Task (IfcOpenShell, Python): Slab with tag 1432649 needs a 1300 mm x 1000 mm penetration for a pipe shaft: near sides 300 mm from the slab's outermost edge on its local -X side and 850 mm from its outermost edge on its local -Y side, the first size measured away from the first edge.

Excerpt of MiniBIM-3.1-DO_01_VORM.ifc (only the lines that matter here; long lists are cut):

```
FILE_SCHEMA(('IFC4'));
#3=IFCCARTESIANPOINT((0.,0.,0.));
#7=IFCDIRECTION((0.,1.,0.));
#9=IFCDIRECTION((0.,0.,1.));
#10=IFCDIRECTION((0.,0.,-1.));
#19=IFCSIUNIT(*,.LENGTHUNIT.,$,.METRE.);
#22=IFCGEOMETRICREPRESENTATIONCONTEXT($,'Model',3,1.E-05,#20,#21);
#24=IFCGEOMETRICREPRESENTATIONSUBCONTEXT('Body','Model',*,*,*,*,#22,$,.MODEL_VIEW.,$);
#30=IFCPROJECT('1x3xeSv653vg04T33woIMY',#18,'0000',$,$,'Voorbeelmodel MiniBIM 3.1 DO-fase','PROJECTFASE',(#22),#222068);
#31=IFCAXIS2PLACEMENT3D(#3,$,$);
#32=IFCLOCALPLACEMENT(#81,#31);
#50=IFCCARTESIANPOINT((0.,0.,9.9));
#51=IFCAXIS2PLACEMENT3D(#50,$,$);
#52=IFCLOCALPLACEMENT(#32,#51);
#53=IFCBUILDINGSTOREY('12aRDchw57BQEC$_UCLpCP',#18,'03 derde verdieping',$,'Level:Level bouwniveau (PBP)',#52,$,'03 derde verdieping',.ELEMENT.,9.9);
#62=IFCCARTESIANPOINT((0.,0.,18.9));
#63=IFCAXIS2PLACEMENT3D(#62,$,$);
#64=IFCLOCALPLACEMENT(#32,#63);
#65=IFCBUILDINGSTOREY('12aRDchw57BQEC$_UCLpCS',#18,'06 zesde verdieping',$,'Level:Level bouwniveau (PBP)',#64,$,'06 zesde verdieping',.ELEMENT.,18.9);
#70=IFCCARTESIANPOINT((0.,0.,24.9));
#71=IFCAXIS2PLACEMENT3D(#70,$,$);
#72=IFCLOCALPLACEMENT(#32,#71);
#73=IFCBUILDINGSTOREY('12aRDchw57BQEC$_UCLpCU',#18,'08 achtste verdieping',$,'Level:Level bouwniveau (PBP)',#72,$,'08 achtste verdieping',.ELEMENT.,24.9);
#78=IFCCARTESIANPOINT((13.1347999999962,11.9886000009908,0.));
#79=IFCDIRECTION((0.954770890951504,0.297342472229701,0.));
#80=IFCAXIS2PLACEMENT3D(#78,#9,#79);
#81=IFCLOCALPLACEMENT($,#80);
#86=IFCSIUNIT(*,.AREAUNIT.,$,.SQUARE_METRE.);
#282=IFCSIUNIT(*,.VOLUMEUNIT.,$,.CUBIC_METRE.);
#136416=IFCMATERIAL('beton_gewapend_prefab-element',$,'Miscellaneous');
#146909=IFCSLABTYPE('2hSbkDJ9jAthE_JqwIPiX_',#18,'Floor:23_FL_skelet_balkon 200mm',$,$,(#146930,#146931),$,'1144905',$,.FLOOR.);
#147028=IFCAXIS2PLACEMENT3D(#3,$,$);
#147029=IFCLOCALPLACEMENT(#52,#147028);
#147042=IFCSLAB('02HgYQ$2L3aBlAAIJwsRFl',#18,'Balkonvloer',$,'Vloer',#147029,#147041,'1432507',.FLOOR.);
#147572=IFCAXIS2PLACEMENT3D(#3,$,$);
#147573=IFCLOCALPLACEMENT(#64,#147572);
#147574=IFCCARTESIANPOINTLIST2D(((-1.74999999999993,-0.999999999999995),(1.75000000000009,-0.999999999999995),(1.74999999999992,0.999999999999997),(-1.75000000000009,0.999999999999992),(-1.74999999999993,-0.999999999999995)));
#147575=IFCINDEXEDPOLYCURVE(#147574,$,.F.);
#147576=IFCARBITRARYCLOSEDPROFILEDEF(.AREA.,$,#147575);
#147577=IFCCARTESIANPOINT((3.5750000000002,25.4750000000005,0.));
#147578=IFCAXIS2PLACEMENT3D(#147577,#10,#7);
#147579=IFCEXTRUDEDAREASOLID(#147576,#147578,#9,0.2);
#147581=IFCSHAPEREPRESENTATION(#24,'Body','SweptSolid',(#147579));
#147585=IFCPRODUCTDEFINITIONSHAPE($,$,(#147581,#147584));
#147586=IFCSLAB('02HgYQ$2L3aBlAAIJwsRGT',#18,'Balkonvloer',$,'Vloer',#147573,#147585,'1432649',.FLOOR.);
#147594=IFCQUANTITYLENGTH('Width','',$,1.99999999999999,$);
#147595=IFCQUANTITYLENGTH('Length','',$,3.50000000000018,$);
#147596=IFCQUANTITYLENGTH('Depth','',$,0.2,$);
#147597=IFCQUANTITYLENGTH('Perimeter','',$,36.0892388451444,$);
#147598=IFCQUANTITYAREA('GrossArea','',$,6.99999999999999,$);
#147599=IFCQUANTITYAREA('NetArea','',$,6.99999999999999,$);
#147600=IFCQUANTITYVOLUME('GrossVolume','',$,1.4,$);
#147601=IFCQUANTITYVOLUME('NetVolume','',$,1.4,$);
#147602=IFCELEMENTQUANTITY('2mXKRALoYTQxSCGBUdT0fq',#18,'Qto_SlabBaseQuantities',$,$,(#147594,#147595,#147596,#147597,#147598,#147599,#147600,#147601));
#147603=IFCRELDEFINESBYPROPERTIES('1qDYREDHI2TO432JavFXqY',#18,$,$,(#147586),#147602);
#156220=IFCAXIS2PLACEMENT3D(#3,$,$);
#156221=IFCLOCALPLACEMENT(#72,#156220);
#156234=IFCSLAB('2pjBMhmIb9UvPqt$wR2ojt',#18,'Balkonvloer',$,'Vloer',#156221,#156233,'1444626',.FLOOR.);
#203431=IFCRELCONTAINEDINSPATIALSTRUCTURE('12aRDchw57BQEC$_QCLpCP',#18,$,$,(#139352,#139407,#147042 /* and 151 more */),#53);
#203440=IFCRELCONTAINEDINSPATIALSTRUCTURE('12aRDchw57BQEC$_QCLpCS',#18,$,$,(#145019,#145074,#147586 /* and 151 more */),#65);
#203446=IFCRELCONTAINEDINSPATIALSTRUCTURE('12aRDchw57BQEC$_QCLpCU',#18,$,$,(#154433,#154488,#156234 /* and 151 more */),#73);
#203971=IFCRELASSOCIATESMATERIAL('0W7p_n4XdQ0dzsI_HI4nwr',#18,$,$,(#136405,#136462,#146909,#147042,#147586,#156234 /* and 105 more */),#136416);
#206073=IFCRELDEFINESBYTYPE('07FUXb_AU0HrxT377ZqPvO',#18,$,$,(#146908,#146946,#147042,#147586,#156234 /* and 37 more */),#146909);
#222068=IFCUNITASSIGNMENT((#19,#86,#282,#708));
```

```python
import numpy as np
import ifcopenshell
import ifcopenshell.api.feature
import ifcopenshell.api.geometry
import ifcopenshell.api.pset
import ifcopenshell.api.root
import ifcopenshell.geom
import ifcopenshell.util.element
import ifcopenshell.util.placement
import ifcopenshell.util.representation
import ifcopenshell.util.shape
import ifcopenshell.util.unit

model = ifcopenshell.open("MiniBIM-3.1-DO_01_VORM.ifc")
unit_scale = ifcopenshell.util.unit.calculate_unit_scale(model)
area_scale = ifcopenshell.util.unit.calculate_unit_scale(model, "AREAUNIT")
volume_scale = ifcopenshell.util.unit.calculate_unit_scale(model, "VOLUMEUNIT")
settings = ifcopenshell.geom.settings()


def volume(element):
    """Net volume in cubic metres, openings subtracted."""
    shape = ifcopenshell.geom.create_shape(settings, element)
    return ifcopenshell.util.shape.get_volume(shape.geometry)


slab = model.by_guid("02HgYQ$2L3aBlAAIJwsRGT")
before = volume(slab)

# Extent in the slab's own axes, in metres. The edges named are its -X and -Y sides.
slab_shape = ifcopenshell.geom.create_shape(settings, slab)
vertices = ifcopenshell.util.shape.get_vertices(slab_shape.geometry)
x_min, y_min, bottom = vertices.min(axis=0)
top = vertices[:, 2].max()

opening = ifcopenshell.api.root.create_entity(model, ifc_class="IfcOpeningElement", name="Pipe shaft opening", predefined_type="OPENING")
context = ifcopenshell.util.representation.get_context(model, "Model", "Body", "MODEL_VIEW")
width, depth = 1.3, 1
outline = [(0.0, 0.0), (width, 0.0), (width, depth), (0.0, depth), (0.0, 0.0)]
# Overshoot both faces by 50 mm so the cut is clean.
shape = ifcopenshell.api.geometry.add_slab_representation(
    model, context=context, depth=top - bottom + 0.1, polyline=outline
)
ifcopenshell.api.geometry.assign_representation(model, product=opening, representation=shape)

matrix = ifcopenshell.util.placement.get_local_placement(slab.ObjectPlacement)
matrix[:, 3] = matrix @ np.append(np.array([x_min + 0.3, y_min + 0.85, bottom - 0.05]) / unit_scale, 1.0)
ifcopenshell.api.geometry.edit_object_placement(model, product=opening, matrix=matrix, is_si=False)
ifcopenshell.api.feature.add_feature(model, feature=opening, element=slab)

after = volume(slab)

# Update the slab's stored quantities.
qto = model.by_id(ifcopenshell.util.element.get_pset(slab, "Qto_SlabBaseQuantities", should_inherit=False)["id"])
ifcopenshell.api.pset.edit_qto(model, qto=qto, properties={
    "NetArea": after / (top - bottom) / area_scale,
    "NetVolume": after / volume_scale,
})

print(f"slab volume {before:.3f} -> {after:.3f} m3")

model.write("MiniBIM-3.1-DO_01_VORM_updated.ifc")
```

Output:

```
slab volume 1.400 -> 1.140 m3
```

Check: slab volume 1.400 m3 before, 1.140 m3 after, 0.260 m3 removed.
